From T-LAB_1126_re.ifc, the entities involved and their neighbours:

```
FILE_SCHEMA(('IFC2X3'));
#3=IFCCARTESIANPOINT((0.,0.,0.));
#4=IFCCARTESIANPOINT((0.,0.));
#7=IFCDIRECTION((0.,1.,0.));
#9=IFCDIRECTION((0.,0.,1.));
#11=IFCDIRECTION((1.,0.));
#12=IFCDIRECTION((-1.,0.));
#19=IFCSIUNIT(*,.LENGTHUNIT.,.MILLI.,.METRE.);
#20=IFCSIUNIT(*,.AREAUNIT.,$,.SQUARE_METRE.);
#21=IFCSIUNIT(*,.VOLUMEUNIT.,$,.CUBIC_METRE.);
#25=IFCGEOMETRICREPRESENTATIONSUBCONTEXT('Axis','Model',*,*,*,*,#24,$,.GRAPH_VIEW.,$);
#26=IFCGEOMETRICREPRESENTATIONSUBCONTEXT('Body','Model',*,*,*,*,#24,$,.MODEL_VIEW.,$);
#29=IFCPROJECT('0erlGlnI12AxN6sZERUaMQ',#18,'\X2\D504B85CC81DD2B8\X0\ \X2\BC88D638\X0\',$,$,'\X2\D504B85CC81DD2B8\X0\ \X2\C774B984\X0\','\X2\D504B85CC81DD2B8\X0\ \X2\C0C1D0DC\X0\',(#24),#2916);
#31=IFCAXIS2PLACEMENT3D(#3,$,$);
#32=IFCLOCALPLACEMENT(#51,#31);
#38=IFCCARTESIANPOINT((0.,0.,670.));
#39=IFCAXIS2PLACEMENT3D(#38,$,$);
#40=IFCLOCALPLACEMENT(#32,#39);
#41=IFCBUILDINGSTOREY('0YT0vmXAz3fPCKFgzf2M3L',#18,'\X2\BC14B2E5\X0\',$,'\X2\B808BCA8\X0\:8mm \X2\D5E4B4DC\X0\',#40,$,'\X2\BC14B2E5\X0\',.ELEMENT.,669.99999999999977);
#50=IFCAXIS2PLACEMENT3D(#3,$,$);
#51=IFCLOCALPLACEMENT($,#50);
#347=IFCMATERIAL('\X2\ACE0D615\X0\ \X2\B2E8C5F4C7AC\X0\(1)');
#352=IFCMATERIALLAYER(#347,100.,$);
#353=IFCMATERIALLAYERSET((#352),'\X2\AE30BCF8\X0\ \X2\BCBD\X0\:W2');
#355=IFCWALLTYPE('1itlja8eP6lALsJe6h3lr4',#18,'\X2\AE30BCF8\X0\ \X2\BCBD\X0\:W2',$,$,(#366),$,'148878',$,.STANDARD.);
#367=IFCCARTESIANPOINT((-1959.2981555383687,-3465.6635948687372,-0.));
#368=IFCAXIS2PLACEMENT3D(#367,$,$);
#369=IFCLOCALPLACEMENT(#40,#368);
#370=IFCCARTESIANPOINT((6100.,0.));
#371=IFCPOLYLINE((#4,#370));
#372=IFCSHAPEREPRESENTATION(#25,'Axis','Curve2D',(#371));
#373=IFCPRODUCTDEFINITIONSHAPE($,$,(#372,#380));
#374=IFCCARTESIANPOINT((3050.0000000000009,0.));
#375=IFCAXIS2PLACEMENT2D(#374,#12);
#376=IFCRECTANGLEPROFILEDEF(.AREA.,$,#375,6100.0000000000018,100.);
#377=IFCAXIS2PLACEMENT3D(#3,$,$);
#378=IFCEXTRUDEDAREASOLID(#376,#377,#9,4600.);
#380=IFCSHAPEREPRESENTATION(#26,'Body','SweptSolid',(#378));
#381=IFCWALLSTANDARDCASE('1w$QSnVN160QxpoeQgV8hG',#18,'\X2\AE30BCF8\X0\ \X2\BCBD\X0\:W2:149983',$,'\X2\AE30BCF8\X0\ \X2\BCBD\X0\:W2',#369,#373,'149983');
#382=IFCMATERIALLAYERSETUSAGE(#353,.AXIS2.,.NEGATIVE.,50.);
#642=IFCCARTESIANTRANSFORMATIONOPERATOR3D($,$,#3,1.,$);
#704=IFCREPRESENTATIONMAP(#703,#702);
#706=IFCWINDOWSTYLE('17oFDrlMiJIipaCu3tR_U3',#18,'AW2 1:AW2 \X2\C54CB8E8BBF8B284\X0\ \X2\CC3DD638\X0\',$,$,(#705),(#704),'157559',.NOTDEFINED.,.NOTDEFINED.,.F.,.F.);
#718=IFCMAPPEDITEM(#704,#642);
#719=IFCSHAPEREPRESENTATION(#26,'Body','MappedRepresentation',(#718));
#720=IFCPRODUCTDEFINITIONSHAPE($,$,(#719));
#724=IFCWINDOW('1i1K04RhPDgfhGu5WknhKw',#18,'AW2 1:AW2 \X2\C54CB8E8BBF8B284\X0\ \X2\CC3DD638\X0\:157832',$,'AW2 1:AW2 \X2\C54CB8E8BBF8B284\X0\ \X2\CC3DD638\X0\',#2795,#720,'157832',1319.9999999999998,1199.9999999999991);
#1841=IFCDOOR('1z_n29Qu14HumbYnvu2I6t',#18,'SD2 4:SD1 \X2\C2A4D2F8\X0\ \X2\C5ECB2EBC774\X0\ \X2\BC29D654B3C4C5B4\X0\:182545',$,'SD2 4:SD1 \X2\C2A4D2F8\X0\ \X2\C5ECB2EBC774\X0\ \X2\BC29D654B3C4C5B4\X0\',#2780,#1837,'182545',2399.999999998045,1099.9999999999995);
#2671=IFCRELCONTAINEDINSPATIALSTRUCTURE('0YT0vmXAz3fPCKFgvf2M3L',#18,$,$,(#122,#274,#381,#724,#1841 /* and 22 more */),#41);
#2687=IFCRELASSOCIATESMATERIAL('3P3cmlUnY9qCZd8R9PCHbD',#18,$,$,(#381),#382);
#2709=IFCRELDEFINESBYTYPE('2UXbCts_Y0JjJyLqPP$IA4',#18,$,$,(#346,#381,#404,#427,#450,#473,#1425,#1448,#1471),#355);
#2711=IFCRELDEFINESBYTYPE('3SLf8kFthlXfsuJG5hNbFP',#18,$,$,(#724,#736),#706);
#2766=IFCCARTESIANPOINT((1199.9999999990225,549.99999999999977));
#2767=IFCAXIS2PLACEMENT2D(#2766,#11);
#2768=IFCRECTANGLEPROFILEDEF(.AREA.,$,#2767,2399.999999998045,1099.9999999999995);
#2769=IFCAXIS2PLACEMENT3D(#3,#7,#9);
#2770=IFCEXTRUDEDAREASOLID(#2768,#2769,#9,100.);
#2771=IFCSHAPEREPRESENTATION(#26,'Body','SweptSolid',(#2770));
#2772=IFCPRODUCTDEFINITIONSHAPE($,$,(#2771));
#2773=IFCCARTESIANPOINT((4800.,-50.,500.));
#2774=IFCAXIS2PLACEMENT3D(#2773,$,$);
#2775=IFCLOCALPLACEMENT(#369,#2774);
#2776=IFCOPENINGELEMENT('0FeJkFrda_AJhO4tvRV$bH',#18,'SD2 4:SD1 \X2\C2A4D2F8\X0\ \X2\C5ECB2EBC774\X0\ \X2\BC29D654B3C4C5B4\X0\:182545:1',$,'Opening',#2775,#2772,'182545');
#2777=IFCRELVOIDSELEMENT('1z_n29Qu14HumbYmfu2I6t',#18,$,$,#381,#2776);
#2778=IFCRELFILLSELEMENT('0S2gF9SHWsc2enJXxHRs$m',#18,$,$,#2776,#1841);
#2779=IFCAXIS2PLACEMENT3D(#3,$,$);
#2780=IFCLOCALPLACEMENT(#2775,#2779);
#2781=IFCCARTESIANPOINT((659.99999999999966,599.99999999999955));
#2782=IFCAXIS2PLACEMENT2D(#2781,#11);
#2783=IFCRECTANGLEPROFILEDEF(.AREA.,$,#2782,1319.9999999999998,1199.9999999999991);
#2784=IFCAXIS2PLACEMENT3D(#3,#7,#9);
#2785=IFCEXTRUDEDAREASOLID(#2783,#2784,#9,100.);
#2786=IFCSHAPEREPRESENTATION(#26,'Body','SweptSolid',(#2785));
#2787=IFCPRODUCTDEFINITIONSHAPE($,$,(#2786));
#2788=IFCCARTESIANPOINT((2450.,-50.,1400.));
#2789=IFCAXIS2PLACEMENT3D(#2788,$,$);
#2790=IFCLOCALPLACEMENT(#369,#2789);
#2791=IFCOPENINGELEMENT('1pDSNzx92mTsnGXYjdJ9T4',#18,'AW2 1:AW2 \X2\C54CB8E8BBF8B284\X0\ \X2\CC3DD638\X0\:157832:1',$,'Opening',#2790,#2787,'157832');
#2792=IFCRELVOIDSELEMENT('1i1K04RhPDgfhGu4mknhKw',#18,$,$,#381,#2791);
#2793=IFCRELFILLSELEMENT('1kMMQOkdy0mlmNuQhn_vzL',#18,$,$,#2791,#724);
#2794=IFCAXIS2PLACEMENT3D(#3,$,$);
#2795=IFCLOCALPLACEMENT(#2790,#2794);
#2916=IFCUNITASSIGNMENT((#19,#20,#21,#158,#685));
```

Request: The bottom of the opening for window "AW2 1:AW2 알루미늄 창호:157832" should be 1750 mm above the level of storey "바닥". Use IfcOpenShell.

```python
import numpy as np
import ifcopenshell
import ifcopenshell.api.geometry
import ifcopenshell.geom
import ifcopenshell.util.element
import ifcopenshell.util.placement
import ifcopenshell.util.shape
import ifcopenshell.util.unit

model = ifcopenshell.open("T-LAB_1126_re.ifc")
unit_scale = ifcopenshell.util.unit.calculate_unit_scale(model)

window = model.by_guid("1i1K04RhPDgfhGu5WknhKw")
opening = window.FillsVoids[0].RelatingOpeningElement
storey = ifcopenshell.util.element.get_container(window, ifc_class="IfcBuildingStorey")
level = ifcopenshell.util.placement.get_local_placement(storey.ObjectPlacement)[2, 3]

# The opening's origin need not be at the sill, so measure its lowest point.
shape = ifcopenshell.geom.create_shape(ifcopenshell.geom.settings(), opening)
bottom = ifcopenshell.util.shape.get_shape_bottom_elevation(shape, shape.geometry) / unit_scale
dz = level + 1750.0 - bottom

shift = np.array([0.0, 0.0, dz])
# The window is placed relative to its opening, so it follows when the opening moves.
matrix = ifcopenshell.util.placement.get_local_placement(opening.ObjectPlacement)
matrix[:3, 3] += shift
ifcopenshell.api.geometry.edit_object_placement(
    model, product=opening, matrix=matrix, is_si=False, should_transform_children=True
)

print(f"moved by {dz * unit_scale:+.3f} m")

model.write("T-LAB_1126_re-out.ifc")
```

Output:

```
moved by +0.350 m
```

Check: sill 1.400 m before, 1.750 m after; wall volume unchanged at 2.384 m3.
